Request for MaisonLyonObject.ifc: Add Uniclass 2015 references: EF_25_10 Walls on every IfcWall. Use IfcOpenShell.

First a look at what the model holds.

```python
import ifcopenshell

model = ifcopenshell.open("MaisonLyonObject.ifc")
print(model.schema)
print("classifications:", [c.Name for c in model.by_type("IfcClassification")])
for ifc_class in ("IfcDoor", "IfcRoof", "IfcStair", "IfcWall", "IfcWindow"):
    print(ifc_class, len(model.by_type(ifc_class)))
```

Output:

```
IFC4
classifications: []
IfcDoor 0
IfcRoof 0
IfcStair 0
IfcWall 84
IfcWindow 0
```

```python
import ifcopenshell
import ifcopenshell.api.classification

model = ifcopenshell.open("MaisonLyonObject.ifc")

system = ifcopenshell.api.classification.add_classification(model, classification="Uniclass 2015")

codes = {
    "IfcWall": ("EF_25_10", "Walls"),
}
for ifc_class, (code, name) in codes.items():
    products = model.by_type(ifc_class)
    ifcopenshell.api.classification.add_reference(
        model, products=products, classification=system, identification=code, name=name
    )
    print(code, len(products))

model.write("MaisonLyonObject_rev.ifc")
```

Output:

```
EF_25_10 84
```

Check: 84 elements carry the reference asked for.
